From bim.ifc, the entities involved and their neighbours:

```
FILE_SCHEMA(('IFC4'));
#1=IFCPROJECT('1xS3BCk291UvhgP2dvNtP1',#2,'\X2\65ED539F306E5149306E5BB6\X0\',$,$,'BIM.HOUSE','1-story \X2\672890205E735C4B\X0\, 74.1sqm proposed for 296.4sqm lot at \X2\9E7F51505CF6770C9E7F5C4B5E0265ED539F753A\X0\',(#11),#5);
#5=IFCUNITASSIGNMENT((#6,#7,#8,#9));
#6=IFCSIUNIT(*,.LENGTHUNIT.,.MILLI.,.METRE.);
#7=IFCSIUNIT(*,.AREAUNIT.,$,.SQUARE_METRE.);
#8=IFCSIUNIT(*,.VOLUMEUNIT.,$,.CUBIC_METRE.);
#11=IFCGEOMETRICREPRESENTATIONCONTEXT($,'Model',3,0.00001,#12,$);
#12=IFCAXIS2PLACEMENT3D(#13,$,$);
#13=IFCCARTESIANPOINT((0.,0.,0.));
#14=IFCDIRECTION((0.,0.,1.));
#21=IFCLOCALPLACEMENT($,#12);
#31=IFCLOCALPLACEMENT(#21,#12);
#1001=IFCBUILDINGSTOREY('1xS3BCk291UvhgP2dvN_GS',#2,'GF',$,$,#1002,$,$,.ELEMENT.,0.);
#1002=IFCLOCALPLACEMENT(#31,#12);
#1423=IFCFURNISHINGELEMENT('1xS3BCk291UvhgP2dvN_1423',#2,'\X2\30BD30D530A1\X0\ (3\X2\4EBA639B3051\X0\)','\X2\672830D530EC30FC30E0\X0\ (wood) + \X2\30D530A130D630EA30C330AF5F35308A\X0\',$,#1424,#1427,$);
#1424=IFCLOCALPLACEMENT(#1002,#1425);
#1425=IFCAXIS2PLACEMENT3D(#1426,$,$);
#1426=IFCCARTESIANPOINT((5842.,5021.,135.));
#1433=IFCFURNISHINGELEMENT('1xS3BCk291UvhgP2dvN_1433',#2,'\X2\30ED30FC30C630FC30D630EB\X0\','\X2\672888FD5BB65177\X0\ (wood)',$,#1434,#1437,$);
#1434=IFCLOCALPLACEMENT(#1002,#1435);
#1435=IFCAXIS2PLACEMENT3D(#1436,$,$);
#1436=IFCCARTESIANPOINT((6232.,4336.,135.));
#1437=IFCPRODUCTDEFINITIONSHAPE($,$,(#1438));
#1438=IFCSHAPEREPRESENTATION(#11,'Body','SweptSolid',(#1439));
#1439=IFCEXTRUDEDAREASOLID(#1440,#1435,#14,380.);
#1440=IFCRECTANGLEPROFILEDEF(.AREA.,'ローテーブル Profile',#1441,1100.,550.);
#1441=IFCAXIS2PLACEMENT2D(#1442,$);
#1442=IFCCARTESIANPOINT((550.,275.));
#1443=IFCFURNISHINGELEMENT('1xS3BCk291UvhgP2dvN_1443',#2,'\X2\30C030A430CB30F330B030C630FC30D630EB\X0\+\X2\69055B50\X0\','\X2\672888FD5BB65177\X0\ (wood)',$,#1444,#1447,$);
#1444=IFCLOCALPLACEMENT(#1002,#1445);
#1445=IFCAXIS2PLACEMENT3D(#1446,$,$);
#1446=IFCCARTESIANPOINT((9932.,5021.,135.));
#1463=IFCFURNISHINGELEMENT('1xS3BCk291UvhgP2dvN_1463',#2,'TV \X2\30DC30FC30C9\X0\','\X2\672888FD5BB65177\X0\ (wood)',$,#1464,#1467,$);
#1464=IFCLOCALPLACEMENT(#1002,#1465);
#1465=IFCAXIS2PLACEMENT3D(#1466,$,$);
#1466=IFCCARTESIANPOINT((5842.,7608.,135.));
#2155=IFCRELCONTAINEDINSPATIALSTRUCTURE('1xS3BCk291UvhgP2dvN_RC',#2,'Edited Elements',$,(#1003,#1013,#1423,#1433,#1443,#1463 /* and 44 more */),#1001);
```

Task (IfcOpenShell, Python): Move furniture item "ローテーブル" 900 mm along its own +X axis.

```python
import ifcopenshell
import ifcopenshell.api.geometry
import ifcopenshell.util.placement

model = ifcopenshell.open("bim.ifc")

item = model.by_guid("1xS3BCk291UvhgP2dvN_1433")
matrix = ifcopenshell.util.placement.get_local_placement(item.ObjectPlacement)
matrix[:3, 3] += matrix[:3, 0] * 900.0
ifcopenshell.api.geometry.edit_object_placement(model, product=item, matrix=matrix, is_si=False)

print(ifcopenshell.util.placement.get_local_placement(item.ObjectPlacement).round(3) + 0.0)

model.write("bim-out.ifc")
```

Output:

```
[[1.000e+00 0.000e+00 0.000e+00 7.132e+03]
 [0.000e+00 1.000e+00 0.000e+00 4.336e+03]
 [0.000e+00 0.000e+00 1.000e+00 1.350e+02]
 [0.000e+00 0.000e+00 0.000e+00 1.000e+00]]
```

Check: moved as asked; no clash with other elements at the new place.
